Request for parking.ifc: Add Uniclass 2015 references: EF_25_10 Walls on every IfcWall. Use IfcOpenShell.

First a look at what the model holds.

```python
import ifcopenshell

model = ifcopenshell.open("parking.ifc")
print(model.schema)
print("classifications:", [c.Name for c in model.by_type("IfcClassification")])
for ifc_class in ("IfcDoor", "IfcRoof", "IfcStair", "IfcWall", "IfcWindow"):
    print(ifc_class, len(model.by_type(ifc_class)))
```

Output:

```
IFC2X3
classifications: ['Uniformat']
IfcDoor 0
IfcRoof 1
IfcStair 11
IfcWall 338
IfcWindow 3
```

```python
import ifcopenshell
import ifcopenshell.api.classification

model = ifcopenshell.open("parking.ifc")

# IFC2X3 requires Source and Edition and has no link from the project to the system.
system = model.create_entity("IfcClassification", Source="NBS", Edition="2015", Name="Uniclass 2015")

codes = {
    "IfcWall": ("EF_25_10", "Walls"),
}
for ifc_class, (code, name) in codes.items():
    products = model.by_type(ifc_class)
    ifcopenshell.api.classification.add_reference(
        model, products=products, classification=system, identification=code, name=name
    )
    print(code, len(products))

model.write("parking_v2.ifc")
```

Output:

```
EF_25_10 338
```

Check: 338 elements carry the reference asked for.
